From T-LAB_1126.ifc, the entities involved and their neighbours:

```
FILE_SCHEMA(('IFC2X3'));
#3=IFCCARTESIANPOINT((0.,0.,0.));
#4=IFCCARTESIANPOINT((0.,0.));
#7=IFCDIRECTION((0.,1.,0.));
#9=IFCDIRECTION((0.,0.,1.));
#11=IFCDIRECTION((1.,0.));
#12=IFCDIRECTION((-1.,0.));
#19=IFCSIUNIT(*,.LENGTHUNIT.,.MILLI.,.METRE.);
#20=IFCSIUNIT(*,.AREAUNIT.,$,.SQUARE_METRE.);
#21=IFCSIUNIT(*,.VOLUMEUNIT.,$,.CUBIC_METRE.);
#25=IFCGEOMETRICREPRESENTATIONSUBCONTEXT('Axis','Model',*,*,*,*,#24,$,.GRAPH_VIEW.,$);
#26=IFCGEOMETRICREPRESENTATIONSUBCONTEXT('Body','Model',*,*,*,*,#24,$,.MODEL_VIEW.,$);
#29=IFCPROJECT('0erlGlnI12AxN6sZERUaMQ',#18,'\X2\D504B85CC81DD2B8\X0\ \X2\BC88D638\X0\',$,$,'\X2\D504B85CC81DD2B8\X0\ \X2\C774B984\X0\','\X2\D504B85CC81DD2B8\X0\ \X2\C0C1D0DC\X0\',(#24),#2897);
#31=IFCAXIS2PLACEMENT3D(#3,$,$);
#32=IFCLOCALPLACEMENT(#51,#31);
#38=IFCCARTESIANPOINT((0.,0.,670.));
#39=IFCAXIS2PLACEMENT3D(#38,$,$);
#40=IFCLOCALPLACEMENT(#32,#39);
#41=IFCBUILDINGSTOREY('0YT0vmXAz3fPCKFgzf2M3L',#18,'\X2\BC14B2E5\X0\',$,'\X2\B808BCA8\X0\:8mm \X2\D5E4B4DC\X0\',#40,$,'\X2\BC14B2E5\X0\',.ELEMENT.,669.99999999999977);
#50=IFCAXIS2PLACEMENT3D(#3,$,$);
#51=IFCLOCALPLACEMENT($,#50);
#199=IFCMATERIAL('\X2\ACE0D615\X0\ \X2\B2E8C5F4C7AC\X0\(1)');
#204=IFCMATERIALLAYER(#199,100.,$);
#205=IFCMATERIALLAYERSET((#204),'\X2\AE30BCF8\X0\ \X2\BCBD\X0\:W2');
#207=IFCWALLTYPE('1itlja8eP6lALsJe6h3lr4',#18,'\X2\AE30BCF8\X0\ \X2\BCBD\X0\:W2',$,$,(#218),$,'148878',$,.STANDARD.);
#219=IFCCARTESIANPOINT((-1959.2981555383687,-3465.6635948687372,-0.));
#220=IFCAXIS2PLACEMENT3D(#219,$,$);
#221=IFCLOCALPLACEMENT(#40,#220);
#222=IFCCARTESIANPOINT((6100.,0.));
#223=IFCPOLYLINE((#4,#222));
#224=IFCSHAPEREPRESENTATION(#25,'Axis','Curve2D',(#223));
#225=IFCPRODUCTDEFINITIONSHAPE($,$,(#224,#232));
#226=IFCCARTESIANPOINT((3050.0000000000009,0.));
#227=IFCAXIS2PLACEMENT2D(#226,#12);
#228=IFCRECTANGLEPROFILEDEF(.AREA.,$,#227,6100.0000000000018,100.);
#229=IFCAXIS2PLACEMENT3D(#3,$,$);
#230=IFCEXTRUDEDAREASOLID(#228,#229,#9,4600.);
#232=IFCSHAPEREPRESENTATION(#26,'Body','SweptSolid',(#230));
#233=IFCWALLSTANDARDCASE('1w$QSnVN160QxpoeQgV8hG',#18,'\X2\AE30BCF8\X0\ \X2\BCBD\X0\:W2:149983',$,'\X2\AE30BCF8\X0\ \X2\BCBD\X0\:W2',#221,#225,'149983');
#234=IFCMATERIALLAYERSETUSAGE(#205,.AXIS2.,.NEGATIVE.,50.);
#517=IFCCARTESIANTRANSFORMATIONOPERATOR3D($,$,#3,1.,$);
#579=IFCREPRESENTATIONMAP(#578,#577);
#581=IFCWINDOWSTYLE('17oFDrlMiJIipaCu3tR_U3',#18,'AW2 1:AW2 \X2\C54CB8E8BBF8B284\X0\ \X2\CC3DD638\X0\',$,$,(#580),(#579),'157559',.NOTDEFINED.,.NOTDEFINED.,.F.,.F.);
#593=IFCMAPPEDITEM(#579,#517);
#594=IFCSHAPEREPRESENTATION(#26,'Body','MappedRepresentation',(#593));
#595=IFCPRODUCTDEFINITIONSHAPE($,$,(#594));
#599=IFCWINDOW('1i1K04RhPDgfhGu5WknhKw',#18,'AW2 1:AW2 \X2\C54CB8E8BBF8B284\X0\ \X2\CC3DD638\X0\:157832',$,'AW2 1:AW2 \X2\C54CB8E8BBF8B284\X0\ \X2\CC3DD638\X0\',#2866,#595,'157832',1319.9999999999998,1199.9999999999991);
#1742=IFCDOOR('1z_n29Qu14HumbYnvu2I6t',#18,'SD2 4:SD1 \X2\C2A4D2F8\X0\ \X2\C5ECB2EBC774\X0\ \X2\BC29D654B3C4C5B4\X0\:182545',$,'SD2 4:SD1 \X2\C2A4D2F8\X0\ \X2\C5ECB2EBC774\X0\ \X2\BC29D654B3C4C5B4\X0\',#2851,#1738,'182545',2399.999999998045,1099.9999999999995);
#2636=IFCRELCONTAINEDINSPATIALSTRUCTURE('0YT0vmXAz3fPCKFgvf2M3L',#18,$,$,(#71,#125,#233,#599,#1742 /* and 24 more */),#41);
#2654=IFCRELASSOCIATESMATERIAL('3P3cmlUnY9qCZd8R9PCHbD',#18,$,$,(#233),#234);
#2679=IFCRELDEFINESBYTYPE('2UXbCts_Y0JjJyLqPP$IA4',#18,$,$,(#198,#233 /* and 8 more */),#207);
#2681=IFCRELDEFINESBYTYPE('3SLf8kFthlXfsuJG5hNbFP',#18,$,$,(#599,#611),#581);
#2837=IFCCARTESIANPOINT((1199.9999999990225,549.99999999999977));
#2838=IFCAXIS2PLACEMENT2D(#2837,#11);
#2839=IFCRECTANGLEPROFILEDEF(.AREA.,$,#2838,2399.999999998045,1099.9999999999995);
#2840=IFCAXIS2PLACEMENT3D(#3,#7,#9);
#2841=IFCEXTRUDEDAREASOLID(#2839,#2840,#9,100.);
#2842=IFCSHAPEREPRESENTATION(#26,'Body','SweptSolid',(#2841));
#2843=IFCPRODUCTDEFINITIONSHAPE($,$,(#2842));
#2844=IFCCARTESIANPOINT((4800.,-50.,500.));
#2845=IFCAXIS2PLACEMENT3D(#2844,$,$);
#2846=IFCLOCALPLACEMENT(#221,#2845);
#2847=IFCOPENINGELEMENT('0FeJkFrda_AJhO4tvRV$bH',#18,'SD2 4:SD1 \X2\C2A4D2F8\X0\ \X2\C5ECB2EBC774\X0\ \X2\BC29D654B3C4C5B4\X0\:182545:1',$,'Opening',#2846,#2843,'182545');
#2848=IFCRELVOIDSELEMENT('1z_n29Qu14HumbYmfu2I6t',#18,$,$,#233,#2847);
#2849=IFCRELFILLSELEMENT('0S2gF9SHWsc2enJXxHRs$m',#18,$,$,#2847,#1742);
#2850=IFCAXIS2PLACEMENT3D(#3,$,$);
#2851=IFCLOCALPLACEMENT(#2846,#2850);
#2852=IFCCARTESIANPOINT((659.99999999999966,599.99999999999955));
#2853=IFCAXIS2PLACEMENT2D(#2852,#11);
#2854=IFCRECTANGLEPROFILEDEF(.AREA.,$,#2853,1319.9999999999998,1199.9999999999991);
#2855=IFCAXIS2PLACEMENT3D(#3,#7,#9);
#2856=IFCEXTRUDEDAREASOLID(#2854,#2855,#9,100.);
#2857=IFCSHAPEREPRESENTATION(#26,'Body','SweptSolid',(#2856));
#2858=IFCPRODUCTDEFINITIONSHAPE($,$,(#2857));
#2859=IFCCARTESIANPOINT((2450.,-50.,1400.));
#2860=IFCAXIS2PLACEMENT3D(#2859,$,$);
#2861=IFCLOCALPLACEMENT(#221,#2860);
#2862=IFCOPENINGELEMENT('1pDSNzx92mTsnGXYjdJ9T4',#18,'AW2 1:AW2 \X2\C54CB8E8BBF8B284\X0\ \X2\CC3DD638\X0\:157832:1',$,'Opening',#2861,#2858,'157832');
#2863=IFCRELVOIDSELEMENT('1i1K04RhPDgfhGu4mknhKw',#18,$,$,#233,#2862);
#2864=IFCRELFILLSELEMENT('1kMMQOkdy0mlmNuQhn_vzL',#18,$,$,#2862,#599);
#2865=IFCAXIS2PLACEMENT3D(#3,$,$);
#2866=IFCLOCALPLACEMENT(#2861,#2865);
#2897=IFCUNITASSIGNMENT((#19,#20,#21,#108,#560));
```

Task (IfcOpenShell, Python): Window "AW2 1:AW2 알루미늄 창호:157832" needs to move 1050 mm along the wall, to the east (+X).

```python
import ifcopenshell
import ifcopenshell.api.geometry
import ifcopenshell.util.placement
import ifcopenshell.util.unit

model = ifcopenshell.open("T-LAB_1126.ifc")
unit_scale = ifcopenshell.util.unit.calculate_unit_scale(model)

window = model.by_guid("1i1K04RhPDgfhGu5WknhKw")
opening = window.FillsVoids[0].RelatingOpeningElement
wall = opening.VoidsElements[0].RelatingBuildingElement

wall_matrix = ifcopenshell.util.placement.get_local_placement(wall.ObjectPlacement)
shift = wall_matrix[:3, 0] * 1.05 / unit_scale
before = ifcopenshell.util.placement.get_local_placement(window.ObjectPlacement)[:3, 3].copy()

# The window is placed relative to its opening, so it follows when the opening moves.
matrix = ifcopenshell.util.placement.get_local_placement(opening.ObjectPlacement)
matrix[:3, 3] += shift
ifcopenshell.api.geometry.edit_object_placement(
    model, product=opening, matrix=matrix, is_si=False, should_transform_children=True
)

after = ifcopenshell.util.placement.get_local_placement(window.ObjectPlacement)[:3, 3]
print("window moved by", (after - before).round(3) + 0.0)

model.write("T-LAB_1126_edited.ifc")
```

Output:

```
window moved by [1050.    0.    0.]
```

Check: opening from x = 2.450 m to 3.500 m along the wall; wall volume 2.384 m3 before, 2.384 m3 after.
